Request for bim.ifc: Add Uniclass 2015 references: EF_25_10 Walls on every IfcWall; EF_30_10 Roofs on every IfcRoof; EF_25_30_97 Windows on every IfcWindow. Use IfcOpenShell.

First a look at what the model holds.

```python
import ifcopenshell

model = ifcopenshell.open("bim.ifc")
print(model.schema)
print("classifications:", [c.Name for c in model.by_type("IfcClassification")])
for ifc_class in ("IfcDoor", "IfcRoof", "IfcStair", "IfcWall", "IfcWindow"):
    print(ifc_class, len(model.by_type(ifc_class)))
```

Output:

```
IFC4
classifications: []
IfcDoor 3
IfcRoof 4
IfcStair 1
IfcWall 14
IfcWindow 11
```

```python
import ifcopenshell
import ifcopenshell.api.classification

model = ifcopenshell.open("bim.ifc")

system = ifcopenshell.api.classification.add_classification(model, classification="Uniclass 2015")

codes = {
    "IfcWall": ("EF_25_10", "Walls"),
    "IfcRoof": ("EF_30_10", "Roofs"),
    "IfcWindow": ("EF_25_30_97", "Windows"),
}
for ifc_class, (code, name) in codes.items():
    products = model.by_type(ifc_class)
    ifcopenshell.api.classification.add_reference(
        model, products=products, classification=system, identification=code, name=name
    )
    print(code, len(products))

model.write("bim-out.ifc")
```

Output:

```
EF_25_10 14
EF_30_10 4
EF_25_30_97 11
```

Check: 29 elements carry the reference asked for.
